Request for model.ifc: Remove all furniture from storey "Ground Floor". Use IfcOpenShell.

First a look at what the model holds.

```python
import ifcopenshell
import ifcopenshell.util.element

model = ifcopenshell.open("model.ifc")
print(model.schema)
storey = next(s for s in model.by_type("IfcBuildingStorey") if s.Name == "Ground Floor")
furniture = [e for e in ifcopenshell.util.element.get_decomposition(storey) if e.is_a("IfcFurnishingElement")]
seen = {}
for e in furniture:
    element_type = ifcopenshell.util.element.get_type(e)
    name = element_type.Name if element_type not in (None, e) else None
    seen[name] = seen.get(name, 0) + 1
for name, count in sorted(seen.items(), key=str):
    print(count, "x", name)
```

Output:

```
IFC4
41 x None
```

```python
import ifcopenshell
import ifcopenshell.api.root
import ifcopenshell.util.element

model = ifcopenshell.open("model.ifc")

storey = next(s for s in model.by_type("IfcBuildingStorey") if s.Name == "Ground Floor")
furniture = [e for e in ifcopenshell.util.element.get_decomposition(storey) if e.is_a("IfcFurnishingElement")]

for e in furniture:
    ifcopenshell.api.root.remove_product(model, product=e)
print(len(furniture), "removed")

model.write("model_updated.ifc")
```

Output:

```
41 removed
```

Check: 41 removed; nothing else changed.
